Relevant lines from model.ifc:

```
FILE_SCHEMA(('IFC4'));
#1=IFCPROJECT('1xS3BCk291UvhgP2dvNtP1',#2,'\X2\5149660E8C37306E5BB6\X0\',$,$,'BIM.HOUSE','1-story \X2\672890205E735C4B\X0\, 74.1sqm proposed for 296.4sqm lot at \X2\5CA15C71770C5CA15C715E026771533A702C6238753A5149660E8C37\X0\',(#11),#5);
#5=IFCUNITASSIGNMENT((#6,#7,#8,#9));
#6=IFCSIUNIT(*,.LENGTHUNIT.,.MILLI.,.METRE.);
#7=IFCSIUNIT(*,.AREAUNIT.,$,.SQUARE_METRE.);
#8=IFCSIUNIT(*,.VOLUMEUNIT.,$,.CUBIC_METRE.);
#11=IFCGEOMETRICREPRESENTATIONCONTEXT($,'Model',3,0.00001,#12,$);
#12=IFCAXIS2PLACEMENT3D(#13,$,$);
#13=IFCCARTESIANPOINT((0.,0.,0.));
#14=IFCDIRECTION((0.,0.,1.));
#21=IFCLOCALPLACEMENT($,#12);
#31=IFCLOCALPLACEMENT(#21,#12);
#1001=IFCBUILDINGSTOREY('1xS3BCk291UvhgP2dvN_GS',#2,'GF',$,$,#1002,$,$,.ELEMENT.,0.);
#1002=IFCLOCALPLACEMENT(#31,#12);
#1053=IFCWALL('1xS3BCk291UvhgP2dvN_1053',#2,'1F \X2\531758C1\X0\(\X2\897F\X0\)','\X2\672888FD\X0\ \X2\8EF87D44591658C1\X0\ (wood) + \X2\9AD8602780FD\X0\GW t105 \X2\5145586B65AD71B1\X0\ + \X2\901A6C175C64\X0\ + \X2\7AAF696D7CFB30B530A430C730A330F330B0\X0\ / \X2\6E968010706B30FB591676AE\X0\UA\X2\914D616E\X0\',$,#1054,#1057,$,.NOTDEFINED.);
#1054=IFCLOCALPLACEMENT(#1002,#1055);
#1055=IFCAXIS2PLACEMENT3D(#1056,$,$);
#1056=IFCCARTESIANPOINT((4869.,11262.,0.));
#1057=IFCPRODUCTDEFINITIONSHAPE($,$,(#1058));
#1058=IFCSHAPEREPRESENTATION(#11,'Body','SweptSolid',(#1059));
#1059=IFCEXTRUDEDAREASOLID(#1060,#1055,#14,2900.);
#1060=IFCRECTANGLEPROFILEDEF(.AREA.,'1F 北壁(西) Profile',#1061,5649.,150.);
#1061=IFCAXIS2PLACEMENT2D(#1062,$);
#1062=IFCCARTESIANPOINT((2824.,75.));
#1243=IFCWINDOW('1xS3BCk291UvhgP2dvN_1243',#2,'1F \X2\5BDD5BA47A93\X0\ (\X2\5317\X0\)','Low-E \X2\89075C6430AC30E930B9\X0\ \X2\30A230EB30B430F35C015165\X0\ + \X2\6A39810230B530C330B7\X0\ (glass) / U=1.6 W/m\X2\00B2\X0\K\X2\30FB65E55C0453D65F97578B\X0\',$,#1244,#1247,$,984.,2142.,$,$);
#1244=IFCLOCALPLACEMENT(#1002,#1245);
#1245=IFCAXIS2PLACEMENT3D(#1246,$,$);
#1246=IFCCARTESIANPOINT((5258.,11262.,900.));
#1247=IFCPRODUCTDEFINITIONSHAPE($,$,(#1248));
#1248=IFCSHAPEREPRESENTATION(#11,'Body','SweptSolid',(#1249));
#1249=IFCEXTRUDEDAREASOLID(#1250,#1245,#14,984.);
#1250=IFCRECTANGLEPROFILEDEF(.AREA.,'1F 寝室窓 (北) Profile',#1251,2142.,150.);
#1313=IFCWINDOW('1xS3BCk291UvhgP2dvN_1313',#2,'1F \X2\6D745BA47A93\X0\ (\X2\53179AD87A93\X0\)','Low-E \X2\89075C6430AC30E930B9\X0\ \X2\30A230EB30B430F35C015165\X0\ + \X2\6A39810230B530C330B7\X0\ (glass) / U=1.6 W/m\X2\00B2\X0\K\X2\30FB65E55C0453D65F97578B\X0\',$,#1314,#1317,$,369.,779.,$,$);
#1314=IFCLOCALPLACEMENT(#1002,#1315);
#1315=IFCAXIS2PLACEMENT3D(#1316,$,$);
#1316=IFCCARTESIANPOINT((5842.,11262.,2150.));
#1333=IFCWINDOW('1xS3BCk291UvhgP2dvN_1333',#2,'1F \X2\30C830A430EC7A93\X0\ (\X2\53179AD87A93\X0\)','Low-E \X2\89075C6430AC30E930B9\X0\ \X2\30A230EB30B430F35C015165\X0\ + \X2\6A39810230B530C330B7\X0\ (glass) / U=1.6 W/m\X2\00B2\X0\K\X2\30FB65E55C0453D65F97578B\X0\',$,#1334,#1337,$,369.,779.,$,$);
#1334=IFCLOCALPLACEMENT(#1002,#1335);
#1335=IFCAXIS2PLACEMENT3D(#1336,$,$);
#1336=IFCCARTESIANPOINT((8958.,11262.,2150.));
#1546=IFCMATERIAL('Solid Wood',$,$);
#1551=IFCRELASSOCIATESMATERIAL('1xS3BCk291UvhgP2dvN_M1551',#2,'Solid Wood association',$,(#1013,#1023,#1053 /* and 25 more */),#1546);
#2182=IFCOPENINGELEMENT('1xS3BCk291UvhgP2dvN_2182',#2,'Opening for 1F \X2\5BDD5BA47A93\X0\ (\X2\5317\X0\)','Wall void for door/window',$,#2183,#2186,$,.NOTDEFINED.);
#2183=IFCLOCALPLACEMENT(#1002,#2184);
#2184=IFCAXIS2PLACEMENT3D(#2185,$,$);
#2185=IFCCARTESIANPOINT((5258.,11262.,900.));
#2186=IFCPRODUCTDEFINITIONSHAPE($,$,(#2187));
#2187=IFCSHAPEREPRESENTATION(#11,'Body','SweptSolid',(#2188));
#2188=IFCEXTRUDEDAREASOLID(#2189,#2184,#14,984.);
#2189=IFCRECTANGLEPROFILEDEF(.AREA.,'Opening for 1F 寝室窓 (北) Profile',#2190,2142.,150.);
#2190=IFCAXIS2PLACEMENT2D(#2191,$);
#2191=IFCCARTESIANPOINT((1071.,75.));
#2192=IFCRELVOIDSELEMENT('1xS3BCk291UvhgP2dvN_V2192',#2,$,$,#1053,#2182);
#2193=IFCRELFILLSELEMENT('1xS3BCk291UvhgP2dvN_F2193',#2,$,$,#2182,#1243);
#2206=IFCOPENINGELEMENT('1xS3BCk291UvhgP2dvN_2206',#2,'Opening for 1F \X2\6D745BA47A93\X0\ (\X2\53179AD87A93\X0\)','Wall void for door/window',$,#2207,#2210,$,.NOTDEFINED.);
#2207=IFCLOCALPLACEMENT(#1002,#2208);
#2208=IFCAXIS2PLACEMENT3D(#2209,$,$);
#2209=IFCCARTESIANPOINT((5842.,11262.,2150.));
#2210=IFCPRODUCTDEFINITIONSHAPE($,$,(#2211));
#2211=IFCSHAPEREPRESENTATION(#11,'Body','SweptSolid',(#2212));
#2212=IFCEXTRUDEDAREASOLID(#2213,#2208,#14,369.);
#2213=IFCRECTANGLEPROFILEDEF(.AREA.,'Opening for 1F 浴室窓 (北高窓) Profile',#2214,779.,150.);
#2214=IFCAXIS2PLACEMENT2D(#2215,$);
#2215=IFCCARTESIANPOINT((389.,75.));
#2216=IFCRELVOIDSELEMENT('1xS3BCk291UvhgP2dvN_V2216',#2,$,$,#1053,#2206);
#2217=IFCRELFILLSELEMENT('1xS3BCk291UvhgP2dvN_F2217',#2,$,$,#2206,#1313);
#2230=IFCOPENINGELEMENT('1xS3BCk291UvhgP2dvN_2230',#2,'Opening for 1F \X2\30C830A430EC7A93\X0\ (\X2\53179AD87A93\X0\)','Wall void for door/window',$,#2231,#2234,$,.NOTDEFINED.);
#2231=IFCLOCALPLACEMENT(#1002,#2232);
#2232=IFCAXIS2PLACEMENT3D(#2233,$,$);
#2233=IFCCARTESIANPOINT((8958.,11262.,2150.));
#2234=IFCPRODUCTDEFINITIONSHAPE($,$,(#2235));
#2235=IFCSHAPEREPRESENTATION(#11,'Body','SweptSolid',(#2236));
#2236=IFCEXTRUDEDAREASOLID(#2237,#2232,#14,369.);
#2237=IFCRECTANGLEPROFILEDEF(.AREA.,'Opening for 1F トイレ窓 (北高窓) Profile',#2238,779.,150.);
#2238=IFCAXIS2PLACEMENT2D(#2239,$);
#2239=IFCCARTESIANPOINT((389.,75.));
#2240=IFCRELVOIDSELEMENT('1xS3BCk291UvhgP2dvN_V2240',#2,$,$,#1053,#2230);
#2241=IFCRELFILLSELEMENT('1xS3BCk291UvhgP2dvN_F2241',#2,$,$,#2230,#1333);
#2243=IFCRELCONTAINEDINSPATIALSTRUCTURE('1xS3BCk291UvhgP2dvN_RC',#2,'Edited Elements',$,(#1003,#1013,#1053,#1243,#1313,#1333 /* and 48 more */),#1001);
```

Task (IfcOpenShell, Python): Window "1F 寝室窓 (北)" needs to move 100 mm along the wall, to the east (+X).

```python
import ifcopenshell
import ifcopenshell.api.geometry
import ifcopenshell.util.placement

model = ifcopenshell.open("model.ifc")

window = model.by_guid("1xS3BCk291UvhgP2dvN_1243")
opening = window.FillsVoids[0].RelatingOpeningElement
wall = opening.VoidsElements[0].RelatingBuildingElement

wall_matrix = ifcopenshell.util.placement.get_local_placement(wall.ObjectPlacement)
shift = wall_matrix[:3, 0] * 100.0
before = ifcopenshell.util.placement.get_local_placement(window.ObjectPlacement)[:3, 3].copy()

# The window is not placed relative to its opening, so move both.
for product in (opening, window):
    matrix = ifcopenshell.util.placement.get_local_placement(product.ObjectPlacement)
    matrix[:3, 3] += shift
    ifcopenshell.api.geometry.edit_object_placement(model, product=product, matrix=matrix, is_si=False)

after = ifcopenshell.util.placement.get_local_placement(window.ObjectPlacement)[:3, 3]
print("window moved by", (after - before).round(3) + 0.0)

model.write("model_rev.ifc")
```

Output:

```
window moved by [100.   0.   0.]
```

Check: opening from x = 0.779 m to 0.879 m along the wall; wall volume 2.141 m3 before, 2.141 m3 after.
